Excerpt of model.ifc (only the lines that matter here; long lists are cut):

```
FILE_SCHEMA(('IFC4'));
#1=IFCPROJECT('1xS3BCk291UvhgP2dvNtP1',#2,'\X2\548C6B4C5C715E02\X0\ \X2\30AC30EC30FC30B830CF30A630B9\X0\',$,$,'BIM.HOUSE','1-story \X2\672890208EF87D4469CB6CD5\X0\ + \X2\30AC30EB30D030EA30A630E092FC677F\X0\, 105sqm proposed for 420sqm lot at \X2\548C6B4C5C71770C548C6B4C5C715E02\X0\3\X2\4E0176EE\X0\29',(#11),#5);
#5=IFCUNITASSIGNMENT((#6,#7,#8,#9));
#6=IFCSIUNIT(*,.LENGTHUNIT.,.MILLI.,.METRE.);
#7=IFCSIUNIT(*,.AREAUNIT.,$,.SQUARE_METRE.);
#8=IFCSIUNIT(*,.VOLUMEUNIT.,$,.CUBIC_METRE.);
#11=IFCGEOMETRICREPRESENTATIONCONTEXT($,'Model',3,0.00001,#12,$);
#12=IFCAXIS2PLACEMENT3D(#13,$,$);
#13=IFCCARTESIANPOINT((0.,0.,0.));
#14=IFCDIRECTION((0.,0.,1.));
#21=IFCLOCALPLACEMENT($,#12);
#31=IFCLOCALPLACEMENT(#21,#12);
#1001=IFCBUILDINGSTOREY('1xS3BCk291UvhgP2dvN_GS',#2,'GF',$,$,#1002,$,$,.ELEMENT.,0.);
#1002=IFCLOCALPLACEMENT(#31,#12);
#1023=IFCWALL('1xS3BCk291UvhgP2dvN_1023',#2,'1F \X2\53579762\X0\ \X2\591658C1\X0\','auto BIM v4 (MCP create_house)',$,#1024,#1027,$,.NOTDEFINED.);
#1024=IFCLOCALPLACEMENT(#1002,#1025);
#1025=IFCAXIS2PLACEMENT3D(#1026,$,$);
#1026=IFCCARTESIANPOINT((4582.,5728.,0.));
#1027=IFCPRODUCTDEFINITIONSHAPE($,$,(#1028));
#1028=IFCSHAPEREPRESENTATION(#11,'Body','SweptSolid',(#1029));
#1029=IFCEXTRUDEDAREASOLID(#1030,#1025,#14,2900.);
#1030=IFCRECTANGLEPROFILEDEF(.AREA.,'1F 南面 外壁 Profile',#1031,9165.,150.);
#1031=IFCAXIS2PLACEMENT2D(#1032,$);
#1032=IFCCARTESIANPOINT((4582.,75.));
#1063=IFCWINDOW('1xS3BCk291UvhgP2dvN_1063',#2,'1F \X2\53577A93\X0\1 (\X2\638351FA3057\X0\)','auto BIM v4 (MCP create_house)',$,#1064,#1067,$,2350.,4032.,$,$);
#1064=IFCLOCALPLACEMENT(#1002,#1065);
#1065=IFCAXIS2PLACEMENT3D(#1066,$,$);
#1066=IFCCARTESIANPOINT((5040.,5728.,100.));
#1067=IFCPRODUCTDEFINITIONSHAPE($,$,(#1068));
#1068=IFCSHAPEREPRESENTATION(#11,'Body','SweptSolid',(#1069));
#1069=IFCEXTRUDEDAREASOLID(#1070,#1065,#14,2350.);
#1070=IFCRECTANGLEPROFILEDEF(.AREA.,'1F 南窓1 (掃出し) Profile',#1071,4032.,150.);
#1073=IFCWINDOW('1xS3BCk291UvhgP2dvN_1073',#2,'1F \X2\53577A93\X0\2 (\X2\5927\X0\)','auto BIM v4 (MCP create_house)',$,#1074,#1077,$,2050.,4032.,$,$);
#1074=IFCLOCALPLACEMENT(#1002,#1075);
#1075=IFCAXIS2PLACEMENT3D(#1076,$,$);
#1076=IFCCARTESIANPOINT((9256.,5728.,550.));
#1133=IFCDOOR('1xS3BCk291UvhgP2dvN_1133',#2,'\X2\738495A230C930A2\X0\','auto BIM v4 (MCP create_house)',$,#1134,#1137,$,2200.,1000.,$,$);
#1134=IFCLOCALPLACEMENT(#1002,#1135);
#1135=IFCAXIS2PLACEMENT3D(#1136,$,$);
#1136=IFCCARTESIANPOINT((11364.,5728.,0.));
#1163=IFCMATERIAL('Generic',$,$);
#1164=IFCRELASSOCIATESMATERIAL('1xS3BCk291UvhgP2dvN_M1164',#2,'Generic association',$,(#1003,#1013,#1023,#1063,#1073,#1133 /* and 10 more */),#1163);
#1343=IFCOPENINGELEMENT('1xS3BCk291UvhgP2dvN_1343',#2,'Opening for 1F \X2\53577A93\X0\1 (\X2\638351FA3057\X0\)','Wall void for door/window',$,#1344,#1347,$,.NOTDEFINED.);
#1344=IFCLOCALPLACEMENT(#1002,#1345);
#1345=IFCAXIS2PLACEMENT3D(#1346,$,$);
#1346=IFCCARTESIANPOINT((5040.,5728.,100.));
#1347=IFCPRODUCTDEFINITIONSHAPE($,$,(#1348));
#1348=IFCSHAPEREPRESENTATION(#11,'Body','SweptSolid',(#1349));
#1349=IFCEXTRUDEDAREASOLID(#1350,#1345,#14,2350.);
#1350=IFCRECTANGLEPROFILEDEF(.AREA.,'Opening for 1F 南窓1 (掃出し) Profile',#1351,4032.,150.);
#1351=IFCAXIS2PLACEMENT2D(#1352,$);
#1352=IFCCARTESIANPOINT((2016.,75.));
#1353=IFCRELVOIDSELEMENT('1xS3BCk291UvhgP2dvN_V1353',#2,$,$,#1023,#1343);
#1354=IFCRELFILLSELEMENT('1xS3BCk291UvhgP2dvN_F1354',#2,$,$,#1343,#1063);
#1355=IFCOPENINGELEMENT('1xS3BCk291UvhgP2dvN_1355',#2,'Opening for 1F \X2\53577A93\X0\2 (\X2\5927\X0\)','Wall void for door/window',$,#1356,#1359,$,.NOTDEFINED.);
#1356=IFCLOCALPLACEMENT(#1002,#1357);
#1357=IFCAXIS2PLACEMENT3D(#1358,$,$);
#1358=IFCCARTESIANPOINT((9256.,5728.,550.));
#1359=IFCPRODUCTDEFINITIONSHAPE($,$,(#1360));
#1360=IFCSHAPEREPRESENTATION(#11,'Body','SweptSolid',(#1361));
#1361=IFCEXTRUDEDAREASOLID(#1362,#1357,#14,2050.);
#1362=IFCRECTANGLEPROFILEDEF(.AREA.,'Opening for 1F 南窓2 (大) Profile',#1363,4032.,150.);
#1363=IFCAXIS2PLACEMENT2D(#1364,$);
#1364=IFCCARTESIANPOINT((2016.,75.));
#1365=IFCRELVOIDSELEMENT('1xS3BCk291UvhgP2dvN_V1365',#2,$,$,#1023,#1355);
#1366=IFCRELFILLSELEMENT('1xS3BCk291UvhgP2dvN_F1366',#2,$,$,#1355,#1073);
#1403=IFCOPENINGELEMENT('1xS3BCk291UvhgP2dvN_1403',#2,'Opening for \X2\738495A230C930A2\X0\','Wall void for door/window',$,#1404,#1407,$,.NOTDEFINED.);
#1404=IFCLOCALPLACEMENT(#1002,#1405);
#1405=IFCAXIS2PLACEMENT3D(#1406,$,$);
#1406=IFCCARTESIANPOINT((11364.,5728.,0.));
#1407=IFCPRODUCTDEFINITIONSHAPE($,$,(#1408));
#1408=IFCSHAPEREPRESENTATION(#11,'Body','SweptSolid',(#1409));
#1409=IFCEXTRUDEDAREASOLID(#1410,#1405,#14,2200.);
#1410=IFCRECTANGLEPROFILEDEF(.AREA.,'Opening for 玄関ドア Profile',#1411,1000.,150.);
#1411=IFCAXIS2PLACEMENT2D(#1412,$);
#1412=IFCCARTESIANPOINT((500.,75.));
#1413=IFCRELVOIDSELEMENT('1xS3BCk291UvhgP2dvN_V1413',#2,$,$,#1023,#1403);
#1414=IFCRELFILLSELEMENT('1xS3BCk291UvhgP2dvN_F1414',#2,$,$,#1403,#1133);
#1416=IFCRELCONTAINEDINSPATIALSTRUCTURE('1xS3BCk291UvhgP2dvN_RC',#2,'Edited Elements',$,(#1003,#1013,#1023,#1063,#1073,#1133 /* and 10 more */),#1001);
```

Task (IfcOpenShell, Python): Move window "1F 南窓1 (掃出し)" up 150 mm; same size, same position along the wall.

```python
import numpy as np
import ifcopenshell
import ifcopenshell.api.geometry
import ifcopenshell.util.placement
import ifcopenshell.util.unit

model = ifcopenshell.open("model.ifc")
unit_scale = ifcopenshell.util.unit.calculate_unit_scale(model)

window = model.by_guid("1xS3BCk291UvhgP2dvN_1063")
opening = window.FillsVoids[0].RelatingOpeningElement
dz = 150.0

shift = np.array([0.0, 0.0, dz])
# The window is not placed relative to its opening, so move both.
for product in (opening, window):
    matrix = ifcopenshell.util.placement.get_local_placement(product.ObjectPlacement)
    matrix[:3, 3] += shift
    ifcopenshell.api.geometry.edit_object_placement(model, product=product, matrix=matrix, is_si=False)

print(f"moved by {dz * unit_scale:+.3f} m")

model.write("model_rev.ifc")
```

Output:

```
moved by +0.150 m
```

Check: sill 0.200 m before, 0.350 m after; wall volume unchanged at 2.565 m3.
